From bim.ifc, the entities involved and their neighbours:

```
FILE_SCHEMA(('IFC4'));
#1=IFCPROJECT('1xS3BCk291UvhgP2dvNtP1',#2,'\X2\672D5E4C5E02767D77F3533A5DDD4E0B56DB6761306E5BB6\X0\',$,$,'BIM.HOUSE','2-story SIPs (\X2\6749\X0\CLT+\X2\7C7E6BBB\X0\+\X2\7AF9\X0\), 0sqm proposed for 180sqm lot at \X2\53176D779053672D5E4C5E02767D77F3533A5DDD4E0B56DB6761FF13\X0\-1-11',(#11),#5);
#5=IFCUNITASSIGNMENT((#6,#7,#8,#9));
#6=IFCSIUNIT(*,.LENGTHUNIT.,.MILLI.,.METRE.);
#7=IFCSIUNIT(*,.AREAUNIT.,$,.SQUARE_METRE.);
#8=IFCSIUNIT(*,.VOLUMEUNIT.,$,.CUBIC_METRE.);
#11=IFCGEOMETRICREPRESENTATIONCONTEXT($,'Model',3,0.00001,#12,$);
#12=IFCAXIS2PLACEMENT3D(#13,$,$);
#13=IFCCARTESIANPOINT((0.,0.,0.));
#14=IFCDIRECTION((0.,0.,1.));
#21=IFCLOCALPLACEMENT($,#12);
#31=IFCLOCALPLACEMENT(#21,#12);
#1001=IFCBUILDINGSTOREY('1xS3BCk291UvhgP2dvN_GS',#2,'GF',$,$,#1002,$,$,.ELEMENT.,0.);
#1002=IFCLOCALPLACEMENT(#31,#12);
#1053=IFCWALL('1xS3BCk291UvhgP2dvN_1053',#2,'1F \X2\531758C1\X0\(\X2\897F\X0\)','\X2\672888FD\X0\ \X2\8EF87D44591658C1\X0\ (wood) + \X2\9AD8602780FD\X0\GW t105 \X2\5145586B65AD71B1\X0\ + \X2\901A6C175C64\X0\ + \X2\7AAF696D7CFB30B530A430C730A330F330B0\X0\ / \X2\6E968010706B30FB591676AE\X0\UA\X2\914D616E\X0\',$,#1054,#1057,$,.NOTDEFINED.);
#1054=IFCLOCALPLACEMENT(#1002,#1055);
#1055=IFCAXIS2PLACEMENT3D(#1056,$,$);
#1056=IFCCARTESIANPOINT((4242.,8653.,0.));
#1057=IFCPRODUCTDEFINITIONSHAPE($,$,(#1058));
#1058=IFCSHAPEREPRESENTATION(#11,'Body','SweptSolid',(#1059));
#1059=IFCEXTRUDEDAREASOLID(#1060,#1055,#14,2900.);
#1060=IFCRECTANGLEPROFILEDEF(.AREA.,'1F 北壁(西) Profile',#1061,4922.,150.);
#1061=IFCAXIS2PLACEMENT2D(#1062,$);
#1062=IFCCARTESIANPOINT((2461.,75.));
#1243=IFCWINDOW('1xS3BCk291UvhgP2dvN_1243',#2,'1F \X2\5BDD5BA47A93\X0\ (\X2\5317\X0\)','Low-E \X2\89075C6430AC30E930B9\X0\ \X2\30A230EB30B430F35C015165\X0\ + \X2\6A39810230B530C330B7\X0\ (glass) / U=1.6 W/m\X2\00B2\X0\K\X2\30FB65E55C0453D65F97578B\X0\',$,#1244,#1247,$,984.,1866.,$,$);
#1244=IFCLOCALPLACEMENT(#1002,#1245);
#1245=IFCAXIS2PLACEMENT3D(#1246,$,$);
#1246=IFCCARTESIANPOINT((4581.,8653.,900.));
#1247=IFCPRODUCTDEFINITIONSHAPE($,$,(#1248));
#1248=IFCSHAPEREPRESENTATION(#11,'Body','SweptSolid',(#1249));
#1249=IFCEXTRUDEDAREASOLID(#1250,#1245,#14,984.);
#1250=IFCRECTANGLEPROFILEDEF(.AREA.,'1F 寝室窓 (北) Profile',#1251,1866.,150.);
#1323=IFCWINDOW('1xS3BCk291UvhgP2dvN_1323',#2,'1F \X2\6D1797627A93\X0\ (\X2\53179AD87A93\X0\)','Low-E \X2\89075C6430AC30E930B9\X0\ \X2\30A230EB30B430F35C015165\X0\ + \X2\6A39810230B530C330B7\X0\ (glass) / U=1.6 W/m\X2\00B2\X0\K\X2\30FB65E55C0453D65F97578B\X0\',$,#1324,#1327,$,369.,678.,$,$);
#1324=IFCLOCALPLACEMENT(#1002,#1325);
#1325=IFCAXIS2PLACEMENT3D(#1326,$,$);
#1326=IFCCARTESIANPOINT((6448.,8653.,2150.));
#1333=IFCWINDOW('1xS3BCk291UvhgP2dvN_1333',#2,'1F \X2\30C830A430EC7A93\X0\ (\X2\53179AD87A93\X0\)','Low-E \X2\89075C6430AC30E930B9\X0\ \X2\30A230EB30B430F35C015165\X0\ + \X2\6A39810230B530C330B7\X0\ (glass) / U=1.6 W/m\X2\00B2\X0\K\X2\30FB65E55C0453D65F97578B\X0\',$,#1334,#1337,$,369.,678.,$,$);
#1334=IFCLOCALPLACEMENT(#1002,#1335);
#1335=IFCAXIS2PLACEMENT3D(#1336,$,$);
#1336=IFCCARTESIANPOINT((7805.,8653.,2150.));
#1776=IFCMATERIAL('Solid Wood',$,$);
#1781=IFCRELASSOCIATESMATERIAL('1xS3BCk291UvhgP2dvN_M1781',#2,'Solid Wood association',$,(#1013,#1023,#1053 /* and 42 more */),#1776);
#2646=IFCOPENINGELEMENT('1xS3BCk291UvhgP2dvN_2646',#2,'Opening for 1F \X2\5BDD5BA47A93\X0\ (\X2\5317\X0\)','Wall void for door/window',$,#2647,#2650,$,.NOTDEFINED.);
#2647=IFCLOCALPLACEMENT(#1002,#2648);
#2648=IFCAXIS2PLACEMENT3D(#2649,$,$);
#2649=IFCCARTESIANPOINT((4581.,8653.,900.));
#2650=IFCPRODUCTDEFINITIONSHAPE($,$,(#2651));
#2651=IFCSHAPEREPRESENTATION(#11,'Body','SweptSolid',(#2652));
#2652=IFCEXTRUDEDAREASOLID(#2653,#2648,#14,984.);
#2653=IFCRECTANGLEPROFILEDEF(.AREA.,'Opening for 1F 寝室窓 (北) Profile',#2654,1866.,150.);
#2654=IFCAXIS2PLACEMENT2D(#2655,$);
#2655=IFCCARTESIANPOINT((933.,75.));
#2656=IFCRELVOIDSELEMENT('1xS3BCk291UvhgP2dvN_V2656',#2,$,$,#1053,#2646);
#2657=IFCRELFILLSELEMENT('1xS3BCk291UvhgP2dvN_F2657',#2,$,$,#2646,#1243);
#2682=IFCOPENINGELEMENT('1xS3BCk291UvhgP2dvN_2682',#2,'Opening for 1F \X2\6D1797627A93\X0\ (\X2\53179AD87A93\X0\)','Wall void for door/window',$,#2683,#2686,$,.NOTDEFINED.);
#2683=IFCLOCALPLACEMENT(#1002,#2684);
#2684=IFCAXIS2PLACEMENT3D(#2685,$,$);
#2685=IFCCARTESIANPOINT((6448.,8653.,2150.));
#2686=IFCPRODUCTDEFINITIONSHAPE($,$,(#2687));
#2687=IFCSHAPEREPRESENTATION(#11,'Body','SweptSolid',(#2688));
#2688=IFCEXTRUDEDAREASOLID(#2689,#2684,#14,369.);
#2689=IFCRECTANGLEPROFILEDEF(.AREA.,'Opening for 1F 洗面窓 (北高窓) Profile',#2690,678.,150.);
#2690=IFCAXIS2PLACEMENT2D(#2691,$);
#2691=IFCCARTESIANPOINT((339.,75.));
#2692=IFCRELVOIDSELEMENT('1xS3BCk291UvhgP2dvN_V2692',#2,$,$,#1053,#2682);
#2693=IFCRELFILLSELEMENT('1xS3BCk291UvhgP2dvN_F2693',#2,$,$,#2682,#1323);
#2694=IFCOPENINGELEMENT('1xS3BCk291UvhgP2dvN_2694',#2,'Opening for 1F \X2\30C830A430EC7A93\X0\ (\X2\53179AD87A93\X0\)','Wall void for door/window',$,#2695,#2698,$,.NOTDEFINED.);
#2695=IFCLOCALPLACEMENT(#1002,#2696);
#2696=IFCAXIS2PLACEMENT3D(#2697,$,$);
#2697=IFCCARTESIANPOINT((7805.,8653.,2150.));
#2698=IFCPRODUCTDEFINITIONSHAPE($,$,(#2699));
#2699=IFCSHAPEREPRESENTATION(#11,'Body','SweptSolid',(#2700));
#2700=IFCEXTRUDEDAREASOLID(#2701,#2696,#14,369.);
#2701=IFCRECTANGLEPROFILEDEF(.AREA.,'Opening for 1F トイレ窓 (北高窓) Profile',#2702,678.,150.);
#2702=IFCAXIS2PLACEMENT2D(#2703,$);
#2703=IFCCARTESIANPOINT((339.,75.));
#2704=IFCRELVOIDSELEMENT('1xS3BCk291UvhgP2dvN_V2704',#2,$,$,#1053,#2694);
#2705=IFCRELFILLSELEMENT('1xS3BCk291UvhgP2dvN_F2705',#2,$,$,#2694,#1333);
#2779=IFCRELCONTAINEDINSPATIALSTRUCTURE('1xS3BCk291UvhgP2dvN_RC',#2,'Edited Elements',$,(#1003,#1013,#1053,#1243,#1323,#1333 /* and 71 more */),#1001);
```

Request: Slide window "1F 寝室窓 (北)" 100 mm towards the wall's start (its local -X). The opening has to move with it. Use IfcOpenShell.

```python
import ifcopenshell
import ifcopenshell.api.geometry
import ifcopenshell.util.placement

model = ifcopenshell.open("bim.ifc")

window = model.by_guid("1xS3BCk291UvhgP2dvN_1243")
opening = window.FillsVoids[0].RelatingOpeningElement
wall = opening.VoidsElements[0].RelatingBuildingElement

wall_matrix = ifcopenshell.util.placement.get_local_placement(wall.ObjectPlacement)
shift = wall_matrix[:3, 0] * -100.0
before = ifcopenshell.util.placement.get_local_placement(window.ObjectPlacement)[:3, 3].copy()

# The window is not placed relative to its opening, so move both.
for product in (opening, window):
    matrix = ifcopenshell.util.placement.get_local_placement(product.ObjectPlacement)
    matrix[:3, 3] += shift
    ifcopenshell.api.geometry.edit_object_placement(model, product=product, matrix=matrix, is_si=False)

after = ifcopenshell.util.placement.get_local_placement(window.ObjectPlacement)[:3, 3]
print("window moved by", (after - before).round(3) + 0.0)

model.write("bim_rev.ifc")
```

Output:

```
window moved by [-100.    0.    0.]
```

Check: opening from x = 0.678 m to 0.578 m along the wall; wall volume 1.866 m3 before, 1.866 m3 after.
